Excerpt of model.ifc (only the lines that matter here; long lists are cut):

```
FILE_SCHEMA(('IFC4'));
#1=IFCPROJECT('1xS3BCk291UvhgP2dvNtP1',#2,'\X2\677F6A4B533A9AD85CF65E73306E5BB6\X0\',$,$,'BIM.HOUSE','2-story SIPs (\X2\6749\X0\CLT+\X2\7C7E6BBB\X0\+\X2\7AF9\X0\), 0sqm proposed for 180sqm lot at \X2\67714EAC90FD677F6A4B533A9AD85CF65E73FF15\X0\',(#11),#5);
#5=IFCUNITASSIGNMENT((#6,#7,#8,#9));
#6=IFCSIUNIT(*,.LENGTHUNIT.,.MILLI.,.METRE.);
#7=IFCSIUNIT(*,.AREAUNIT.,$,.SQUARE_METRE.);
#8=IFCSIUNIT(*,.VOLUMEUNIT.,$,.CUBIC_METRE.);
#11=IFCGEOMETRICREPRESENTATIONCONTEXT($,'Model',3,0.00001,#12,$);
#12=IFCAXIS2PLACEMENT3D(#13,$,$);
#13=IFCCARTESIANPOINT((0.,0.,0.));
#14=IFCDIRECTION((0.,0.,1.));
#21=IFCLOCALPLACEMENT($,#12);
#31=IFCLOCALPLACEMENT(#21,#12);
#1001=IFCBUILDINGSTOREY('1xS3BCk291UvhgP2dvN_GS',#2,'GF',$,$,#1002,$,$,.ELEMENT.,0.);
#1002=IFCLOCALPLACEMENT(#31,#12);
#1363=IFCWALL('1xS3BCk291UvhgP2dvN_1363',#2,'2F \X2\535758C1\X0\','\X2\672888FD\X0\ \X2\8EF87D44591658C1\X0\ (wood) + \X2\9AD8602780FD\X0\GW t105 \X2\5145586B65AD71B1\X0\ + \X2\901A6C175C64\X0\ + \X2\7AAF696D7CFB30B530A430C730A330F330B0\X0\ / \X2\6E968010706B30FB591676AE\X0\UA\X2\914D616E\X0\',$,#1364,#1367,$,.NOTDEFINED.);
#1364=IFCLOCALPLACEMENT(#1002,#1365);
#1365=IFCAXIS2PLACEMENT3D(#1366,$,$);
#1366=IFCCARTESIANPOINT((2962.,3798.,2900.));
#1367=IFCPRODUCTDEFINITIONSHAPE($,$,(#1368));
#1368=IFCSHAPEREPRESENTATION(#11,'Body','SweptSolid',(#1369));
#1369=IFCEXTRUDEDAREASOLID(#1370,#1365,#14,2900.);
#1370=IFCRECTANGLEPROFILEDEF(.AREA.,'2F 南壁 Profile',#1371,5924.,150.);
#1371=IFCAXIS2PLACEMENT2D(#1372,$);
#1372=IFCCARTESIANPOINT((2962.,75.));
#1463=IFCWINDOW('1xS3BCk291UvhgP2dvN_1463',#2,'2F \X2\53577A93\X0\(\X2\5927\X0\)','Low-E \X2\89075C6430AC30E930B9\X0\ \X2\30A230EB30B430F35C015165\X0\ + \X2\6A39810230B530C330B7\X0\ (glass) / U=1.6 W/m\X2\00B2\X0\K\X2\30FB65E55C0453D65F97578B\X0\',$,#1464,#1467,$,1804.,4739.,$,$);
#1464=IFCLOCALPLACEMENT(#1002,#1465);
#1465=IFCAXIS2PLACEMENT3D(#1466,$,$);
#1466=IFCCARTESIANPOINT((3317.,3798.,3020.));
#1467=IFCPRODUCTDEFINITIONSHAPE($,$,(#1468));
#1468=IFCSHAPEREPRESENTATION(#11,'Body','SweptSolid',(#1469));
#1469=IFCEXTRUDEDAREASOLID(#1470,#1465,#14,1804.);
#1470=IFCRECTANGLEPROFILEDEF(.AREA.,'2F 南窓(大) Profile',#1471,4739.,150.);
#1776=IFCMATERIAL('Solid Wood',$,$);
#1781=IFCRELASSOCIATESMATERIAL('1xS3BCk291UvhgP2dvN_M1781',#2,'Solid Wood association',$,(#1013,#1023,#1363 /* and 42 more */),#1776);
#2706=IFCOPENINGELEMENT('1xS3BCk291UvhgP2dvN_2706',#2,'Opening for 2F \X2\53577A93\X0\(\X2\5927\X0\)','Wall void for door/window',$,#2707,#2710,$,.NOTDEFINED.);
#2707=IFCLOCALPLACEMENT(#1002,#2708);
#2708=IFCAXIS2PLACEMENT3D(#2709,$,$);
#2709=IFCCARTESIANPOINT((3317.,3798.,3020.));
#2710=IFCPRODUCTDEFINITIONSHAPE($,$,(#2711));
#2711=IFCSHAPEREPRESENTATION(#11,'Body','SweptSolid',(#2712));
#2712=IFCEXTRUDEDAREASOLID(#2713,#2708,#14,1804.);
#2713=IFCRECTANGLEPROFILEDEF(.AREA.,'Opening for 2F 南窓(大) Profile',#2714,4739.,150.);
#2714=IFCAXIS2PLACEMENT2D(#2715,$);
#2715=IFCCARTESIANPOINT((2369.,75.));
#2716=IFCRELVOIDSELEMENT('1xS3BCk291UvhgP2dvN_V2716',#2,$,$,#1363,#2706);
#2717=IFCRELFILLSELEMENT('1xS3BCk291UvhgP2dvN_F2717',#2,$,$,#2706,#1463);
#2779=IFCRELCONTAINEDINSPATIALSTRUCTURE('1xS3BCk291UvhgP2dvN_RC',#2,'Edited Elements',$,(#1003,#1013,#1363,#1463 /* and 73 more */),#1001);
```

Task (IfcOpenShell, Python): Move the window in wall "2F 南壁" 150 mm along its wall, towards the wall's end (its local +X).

```python
import ifcopenshell
import ifcopenshell.api.geometry
import ifcopenshell.util.placement
import ifcopenshell.util.unit

model = ifcopenshell.open("model.ifc")
unit_scale = ifcopenshell.util.unit.calculate_unit_scale(model)

window = model.by_id(1463)
opening = window.FillsVoids[0].RelatingOpeningElement
wall = opening.VoidsElements[0].RelatingBuildingElement

wall_matrix = ifcopenshell.util.placement.get_local_placement(wall.ObjectPlacement)
shift = wall_matrix[:3, 0] * 0.15 / unit_scale
before = ifcopenshell.util.placement.get_local_placement(window.ObjectPlacement)[:3, 3].copy()

# The window is not placed relative to its opening, so move both.
for product in (opening, window):
    matrix = ifcopenshell.util.placement.get_local_placement(product.ObjectPlacement)
    matrix[:3, 3] += shift
    ifcopenshell.api.geometry.edit_object_placement(model, product=product, matrix=matrix, is_si=False)

after = ifcopenshell.util.placement.get_local_placement(window.ObjectPlacement)[:3, 3]
print("window moved by", (after - before).round(3) + 0.0)

model.write("model_rev.ifc")
```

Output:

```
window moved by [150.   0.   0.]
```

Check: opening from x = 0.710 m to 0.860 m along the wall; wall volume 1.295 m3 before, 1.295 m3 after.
